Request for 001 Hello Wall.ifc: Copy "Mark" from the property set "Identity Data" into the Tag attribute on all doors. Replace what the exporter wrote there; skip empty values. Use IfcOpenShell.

First a look at what the model holds.

```python
import ifcopenshell
import ifcopenshell.util.element

model = ifcopenshell.open("001 Hello Wall.ifc")
print(model.schema)
doors = model.by_type("IfcDoor")
print(len(doors), "doors")
for e in doors[:8]:
    source = ifcopenshell.util.element.get_pset(e, "Identity Data", "Mark")
    target = e.Tag
    print(e.id(), repr(source), repr(target), sep=" | ")
```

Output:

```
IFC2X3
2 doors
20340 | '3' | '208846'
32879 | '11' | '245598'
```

```python
import ifcopenshell
import ifcopenshell.util.element

model = ifcopenshell.open("001 Hello Wall.ifc")

count = 0
for e in model.by_type("IfcDoor"):
    value = ifcopenshell.util.element.get_pset(e, "Identity Data", "Mark")
    current = e.Tag
    if not value or not value.strip() or current == value:
        continue
    e.Tag = value
    count += 1

print(count, "doors updated")

model.write("001 Hello Wall_rev.ifc")
```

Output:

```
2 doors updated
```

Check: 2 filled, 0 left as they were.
